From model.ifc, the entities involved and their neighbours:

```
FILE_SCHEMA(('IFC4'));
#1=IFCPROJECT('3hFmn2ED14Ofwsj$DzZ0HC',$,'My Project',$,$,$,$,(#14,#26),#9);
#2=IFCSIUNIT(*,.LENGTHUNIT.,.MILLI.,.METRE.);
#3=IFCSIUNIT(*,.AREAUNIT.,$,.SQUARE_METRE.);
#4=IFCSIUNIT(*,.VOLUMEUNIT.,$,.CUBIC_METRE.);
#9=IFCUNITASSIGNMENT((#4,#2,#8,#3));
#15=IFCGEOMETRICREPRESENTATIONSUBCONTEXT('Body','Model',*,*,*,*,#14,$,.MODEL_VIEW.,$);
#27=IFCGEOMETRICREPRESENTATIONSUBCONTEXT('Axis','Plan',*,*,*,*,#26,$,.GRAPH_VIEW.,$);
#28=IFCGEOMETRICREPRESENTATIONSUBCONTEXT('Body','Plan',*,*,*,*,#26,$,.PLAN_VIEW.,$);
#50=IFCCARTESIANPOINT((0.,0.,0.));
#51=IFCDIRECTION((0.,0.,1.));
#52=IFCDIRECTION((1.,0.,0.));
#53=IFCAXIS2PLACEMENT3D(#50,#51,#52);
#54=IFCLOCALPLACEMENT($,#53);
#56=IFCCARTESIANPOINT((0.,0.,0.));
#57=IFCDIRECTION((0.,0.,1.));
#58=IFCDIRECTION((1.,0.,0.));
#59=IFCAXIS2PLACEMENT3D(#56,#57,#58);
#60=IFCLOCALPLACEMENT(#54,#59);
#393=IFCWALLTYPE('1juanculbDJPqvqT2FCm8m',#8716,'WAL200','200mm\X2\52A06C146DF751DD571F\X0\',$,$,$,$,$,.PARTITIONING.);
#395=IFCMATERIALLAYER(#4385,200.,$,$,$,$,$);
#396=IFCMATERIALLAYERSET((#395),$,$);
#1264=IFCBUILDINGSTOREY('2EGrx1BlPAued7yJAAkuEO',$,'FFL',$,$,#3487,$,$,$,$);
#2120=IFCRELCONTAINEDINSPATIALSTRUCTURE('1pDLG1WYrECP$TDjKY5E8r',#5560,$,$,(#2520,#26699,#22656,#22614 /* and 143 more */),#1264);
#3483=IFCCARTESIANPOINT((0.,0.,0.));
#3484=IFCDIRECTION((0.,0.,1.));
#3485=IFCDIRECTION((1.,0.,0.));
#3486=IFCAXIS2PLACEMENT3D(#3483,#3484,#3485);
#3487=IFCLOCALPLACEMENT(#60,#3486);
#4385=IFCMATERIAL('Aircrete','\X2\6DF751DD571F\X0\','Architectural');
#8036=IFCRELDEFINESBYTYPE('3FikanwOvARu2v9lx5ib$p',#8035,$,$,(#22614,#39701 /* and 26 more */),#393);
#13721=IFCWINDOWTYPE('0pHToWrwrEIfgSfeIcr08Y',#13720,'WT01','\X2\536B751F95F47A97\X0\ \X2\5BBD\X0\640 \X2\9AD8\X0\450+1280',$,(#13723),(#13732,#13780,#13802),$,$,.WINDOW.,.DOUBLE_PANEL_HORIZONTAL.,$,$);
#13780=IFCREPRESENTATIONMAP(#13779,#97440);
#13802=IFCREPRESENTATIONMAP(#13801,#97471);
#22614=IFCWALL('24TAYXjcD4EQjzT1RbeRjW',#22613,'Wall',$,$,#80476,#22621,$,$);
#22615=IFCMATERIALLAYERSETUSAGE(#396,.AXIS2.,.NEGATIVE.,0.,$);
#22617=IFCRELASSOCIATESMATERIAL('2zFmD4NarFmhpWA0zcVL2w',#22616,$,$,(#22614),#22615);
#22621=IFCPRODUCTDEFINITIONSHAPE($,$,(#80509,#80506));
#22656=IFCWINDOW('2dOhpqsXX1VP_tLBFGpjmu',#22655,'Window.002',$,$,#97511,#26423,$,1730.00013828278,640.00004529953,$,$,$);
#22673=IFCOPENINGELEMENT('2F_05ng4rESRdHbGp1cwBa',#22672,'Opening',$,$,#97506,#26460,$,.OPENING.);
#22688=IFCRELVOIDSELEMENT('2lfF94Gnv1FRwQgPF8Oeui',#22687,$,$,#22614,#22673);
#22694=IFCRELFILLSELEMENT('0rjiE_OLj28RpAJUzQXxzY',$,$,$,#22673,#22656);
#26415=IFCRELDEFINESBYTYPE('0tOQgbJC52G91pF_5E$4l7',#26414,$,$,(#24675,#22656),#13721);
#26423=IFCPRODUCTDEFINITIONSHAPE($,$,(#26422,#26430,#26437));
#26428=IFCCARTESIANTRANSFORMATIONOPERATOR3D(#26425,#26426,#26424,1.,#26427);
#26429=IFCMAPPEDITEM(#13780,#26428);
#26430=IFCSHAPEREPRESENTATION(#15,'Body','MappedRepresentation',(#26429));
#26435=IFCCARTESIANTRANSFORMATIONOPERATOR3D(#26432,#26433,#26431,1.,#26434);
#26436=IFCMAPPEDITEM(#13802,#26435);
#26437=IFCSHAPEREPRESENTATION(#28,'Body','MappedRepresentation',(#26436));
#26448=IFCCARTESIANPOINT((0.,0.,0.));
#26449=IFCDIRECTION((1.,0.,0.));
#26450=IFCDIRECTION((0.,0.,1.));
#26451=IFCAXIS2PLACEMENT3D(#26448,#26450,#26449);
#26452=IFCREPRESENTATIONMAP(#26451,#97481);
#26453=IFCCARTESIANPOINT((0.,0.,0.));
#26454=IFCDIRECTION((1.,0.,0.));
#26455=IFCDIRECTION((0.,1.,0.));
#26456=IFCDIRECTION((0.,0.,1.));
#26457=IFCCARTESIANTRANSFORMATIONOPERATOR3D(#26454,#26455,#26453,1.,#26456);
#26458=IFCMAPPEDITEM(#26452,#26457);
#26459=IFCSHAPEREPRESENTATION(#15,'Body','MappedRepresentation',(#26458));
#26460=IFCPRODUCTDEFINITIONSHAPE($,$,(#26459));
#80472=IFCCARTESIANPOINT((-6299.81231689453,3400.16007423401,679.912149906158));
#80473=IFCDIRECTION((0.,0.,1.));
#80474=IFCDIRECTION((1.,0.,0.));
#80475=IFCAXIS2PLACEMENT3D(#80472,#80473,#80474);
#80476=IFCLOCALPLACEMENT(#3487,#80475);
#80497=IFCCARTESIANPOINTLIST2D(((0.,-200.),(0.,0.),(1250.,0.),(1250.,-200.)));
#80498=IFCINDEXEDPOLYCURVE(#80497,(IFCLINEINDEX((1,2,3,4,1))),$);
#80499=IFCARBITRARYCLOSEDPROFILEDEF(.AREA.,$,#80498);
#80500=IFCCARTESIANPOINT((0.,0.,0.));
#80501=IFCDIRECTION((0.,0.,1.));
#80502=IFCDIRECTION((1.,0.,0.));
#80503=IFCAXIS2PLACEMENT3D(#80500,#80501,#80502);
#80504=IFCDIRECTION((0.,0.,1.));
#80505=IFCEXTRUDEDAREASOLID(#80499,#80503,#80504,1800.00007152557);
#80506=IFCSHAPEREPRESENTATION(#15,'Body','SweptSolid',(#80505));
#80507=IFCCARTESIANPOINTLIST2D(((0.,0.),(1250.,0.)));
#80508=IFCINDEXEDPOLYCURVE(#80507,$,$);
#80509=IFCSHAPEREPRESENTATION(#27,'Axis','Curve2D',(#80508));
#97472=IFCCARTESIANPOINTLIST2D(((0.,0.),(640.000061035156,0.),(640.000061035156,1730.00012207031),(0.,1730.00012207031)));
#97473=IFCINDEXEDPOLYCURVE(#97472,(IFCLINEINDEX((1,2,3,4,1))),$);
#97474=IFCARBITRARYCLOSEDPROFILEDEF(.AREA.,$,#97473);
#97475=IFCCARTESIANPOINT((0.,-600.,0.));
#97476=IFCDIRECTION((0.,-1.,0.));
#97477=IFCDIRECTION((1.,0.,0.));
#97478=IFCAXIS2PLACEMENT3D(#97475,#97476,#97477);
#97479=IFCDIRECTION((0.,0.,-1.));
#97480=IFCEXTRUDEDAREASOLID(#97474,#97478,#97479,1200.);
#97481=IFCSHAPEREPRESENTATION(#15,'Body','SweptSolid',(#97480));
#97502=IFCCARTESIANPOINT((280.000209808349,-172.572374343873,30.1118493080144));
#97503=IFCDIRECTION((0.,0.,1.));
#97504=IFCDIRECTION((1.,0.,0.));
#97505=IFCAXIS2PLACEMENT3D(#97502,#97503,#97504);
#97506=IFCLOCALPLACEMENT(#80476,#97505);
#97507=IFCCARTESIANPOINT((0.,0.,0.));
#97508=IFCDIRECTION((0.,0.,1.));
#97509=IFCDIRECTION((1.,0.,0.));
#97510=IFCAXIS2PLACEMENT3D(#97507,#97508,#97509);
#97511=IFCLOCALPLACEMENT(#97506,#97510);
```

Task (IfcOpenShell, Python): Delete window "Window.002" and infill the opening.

```python
import ifcopenshell
import ifcopenshell.api.feature
import ifcopenshell.api.root
import ifcopenshell.geom
import ifcopenshell.util.shape

model = ifcopenshell.open("model.ifc")
settings = ifcopenshell.geom.settings()


def volume(element):
    """Net volume in cubic metres, openings subtracted."""
    shape = ifcopenshell.geom.create_shape(settings, element)
    return ifcopenshell.util.shape.get_volume(shape.geometry)


window = model.by_id(22656)
opening = window.FillsVoids[0].RelatingOpeningElement
wall = opening.VoidsElements[0].RelatingBuildingElement
before = volume(wall)

ifcopenshell.api.root.remove_product(model, product=window)
ifcopenshell.api.feature.remove_feature(model, feature=opening)

after = volume(wall)

print(f"wall volume {before:.3f} -> {after:.3f} m3")

model.write("model_edited.ifc")
```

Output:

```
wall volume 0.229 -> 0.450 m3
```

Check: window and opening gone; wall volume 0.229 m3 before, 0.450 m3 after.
